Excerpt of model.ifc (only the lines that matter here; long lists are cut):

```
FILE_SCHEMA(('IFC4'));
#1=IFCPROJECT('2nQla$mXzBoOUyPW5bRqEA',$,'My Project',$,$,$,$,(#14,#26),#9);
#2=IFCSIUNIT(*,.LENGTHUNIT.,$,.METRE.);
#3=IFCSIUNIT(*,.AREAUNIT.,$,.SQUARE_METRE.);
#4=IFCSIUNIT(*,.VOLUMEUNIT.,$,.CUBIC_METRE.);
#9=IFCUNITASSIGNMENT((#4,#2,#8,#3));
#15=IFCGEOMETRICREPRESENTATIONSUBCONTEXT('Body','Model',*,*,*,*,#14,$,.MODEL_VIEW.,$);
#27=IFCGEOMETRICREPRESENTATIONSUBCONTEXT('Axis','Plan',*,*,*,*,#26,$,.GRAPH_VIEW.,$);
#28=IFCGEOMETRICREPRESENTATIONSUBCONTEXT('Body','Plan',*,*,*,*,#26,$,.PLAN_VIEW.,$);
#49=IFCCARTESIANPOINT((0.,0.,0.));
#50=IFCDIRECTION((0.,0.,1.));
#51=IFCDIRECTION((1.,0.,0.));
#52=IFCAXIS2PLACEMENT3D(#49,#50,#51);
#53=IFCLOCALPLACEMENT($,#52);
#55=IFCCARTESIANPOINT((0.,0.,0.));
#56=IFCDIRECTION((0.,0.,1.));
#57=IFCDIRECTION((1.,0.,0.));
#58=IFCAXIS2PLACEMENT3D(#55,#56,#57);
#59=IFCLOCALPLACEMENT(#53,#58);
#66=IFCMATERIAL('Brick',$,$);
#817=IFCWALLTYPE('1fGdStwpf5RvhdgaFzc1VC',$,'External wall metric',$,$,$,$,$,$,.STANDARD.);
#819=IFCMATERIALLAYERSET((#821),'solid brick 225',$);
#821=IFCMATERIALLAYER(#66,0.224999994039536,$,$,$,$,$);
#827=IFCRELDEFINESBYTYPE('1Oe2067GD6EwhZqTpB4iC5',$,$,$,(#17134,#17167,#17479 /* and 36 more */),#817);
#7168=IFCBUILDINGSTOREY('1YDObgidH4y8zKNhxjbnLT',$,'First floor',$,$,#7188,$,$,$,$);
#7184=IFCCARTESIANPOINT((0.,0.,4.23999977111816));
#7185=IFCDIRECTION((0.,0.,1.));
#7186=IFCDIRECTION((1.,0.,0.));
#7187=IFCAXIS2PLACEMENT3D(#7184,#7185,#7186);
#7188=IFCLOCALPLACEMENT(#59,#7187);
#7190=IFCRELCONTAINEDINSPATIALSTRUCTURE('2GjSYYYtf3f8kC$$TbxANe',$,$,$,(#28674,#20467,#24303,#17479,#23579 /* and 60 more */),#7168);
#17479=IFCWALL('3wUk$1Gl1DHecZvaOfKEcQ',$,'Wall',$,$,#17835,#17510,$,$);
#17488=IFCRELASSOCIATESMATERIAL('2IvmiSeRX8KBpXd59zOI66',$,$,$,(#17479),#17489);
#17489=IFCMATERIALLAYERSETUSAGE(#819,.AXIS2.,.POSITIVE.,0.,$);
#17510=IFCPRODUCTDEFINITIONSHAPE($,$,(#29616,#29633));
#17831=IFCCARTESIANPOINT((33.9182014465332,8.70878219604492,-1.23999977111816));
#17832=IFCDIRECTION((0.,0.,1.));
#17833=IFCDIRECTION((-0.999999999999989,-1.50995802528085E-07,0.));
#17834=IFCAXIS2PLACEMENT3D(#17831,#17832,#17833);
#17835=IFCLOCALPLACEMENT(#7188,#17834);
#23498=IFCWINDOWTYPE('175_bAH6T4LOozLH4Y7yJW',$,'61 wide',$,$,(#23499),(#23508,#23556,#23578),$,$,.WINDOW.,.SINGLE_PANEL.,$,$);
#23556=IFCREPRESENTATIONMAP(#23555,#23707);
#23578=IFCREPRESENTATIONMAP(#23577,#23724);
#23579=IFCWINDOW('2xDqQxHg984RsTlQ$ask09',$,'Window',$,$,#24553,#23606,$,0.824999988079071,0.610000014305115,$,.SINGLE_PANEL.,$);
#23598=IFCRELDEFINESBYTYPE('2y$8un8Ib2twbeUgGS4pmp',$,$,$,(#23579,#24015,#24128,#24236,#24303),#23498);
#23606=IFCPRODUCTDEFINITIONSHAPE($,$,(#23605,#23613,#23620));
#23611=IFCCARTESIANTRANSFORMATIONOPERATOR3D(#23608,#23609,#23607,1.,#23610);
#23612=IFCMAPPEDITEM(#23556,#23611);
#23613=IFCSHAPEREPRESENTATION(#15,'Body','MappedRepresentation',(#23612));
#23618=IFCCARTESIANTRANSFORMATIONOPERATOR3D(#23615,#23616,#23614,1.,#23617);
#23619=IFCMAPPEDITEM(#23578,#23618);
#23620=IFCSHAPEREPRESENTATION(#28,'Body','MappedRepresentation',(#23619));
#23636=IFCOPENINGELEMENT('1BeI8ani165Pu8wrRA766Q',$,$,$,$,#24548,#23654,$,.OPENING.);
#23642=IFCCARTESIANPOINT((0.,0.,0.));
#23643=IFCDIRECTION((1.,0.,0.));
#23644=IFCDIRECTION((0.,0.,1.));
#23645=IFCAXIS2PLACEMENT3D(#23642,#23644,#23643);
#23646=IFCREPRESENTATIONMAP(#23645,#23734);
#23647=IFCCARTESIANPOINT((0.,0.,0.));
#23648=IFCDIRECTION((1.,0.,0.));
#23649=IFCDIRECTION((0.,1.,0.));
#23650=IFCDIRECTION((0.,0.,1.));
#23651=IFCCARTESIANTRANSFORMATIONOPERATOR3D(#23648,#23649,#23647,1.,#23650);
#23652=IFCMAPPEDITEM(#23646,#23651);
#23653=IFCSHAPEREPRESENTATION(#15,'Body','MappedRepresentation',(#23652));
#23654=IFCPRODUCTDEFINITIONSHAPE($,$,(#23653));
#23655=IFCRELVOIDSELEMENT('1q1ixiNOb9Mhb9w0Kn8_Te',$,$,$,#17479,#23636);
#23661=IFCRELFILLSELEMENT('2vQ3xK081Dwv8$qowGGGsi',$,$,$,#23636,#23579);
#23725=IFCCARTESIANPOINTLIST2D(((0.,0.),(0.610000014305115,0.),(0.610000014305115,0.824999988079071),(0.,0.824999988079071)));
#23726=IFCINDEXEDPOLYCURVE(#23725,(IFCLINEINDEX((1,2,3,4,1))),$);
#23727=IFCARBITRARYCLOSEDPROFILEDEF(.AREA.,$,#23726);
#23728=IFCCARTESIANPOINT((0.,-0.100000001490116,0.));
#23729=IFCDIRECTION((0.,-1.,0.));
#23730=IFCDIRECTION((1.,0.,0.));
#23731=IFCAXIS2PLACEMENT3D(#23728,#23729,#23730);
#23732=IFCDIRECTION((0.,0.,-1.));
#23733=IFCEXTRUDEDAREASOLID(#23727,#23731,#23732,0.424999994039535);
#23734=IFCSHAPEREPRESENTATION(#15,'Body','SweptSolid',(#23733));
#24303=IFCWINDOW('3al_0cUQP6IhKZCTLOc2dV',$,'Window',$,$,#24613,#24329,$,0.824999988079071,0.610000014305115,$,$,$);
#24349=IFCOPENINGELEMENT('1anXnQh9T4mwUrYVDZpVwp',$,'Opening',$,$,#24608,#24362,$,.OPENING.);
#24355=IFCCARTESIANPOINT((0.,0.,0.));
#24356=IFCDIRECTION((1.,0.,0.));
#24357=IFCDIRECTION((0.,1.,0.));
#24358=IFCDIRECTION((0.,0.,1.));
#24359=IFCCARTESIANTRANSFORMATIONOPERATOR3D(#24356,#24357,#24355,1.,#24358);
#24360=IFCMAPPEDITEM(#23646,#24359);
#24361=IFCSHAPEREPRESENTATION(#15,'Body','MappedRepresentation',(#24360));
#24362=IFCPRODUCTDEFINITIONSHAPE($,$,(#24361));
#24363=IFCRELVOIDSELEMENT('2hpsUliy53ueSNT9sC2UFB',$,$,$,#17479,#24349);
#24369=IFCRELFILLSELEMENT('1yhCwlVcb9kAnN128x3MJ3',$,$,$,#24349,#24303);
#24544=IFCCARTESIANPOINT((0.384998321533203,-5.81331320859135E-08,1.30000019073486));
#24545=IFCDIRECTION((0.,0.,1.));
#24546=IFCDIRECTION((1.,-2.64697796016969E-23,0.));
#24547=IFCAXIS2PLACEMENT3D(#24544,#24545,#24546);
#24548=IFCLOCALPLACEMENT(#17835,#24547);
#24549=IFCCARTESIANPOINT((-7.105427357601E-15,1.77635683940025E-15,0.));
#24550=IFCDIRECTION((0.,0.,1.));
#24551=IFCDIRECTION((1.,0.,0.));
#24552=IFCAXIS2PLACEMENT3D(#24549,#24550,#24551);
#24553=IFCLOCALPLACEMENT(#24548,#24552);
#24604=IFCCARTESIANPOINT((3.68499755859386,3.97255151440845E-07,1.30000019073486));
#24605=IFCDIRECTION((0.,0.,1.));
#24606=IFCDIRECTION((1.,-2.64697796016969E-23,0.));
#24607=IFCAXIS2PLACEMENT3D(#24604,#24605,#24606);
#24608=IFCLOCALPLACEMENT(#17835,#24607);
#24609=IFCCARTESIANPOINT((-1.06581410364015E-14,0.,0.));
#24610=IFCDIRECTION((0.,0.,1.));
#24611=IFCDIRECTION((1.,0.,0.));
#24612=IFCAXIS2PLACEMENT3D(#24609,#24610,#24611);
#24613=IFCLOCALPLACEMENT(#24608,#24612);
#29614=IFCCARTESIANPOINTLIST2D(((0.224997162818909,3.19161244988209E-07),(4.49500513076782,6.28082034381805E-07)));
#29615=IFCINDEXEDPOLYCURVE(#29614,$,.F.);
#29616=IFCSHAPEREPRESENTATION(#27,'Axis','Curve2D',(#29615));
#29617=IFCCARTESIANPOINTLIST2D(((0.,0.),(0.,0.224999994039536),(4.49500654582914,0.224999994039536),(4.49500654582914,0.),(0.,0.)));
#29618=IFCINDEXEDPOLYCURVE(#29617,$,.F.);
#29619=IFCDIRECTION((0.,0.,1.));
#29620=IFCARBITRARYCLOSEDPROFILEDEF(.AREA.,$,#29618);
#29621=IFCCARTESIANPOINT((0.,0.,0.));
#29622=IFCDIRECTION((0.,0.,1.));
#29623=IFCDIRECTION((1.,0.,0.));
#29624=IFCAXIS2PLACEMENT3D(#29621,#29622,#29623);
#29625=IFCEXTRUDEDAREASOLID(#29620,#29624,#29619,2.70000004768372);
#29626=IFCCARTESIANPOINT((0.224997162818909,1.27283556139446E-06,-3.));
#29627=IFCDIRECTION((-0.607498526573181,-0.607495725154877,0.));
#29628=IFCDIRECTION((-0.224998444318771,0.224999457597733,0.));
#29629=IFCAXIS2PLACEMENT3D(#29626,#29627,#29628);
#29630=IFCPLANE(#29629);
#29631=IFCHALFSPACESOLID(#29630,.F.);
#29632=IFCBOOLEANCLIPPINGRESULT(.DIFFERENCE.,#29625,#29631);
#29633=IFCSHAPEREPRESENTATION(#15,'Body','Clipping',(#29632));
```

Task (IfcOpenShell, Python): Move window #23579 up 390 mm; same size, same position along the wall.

```python
import numpy as np
import ifcopenshell
import ifcopenshell.api.geometry
import ifcopenshell.util.placement
import ifcopenshell.util.unit

model = ifcopenshell.open("model.ifc")
unit_scale = ifcopenshell.util.unit.calculate_unit_scale(model)

window = model.by_id(23579)
opening = window.FillsVoids[0].RelatingOpeningElement
dz = 0.39

shift = np.array([0.0, 0.0, dz])
# The window is placed relative to its opening, so it follows when the opening moves.
matrix = ifcopenshell.util.placement.get_local_placement(opening.ObjectPlacement)
matrix[:3, 3] += shift
ifcopenshell.api.geometry.edit_object_placement(
    model, product=opening, matrix=matrix, is_si=False, should_transform_children=True
)

print(f"moved by {dz * unit_scale:+.3f} m")

model.write("model-out.ifc")
```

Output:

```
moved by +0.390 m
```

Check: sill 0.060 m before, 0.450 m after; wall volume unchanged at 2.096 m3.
